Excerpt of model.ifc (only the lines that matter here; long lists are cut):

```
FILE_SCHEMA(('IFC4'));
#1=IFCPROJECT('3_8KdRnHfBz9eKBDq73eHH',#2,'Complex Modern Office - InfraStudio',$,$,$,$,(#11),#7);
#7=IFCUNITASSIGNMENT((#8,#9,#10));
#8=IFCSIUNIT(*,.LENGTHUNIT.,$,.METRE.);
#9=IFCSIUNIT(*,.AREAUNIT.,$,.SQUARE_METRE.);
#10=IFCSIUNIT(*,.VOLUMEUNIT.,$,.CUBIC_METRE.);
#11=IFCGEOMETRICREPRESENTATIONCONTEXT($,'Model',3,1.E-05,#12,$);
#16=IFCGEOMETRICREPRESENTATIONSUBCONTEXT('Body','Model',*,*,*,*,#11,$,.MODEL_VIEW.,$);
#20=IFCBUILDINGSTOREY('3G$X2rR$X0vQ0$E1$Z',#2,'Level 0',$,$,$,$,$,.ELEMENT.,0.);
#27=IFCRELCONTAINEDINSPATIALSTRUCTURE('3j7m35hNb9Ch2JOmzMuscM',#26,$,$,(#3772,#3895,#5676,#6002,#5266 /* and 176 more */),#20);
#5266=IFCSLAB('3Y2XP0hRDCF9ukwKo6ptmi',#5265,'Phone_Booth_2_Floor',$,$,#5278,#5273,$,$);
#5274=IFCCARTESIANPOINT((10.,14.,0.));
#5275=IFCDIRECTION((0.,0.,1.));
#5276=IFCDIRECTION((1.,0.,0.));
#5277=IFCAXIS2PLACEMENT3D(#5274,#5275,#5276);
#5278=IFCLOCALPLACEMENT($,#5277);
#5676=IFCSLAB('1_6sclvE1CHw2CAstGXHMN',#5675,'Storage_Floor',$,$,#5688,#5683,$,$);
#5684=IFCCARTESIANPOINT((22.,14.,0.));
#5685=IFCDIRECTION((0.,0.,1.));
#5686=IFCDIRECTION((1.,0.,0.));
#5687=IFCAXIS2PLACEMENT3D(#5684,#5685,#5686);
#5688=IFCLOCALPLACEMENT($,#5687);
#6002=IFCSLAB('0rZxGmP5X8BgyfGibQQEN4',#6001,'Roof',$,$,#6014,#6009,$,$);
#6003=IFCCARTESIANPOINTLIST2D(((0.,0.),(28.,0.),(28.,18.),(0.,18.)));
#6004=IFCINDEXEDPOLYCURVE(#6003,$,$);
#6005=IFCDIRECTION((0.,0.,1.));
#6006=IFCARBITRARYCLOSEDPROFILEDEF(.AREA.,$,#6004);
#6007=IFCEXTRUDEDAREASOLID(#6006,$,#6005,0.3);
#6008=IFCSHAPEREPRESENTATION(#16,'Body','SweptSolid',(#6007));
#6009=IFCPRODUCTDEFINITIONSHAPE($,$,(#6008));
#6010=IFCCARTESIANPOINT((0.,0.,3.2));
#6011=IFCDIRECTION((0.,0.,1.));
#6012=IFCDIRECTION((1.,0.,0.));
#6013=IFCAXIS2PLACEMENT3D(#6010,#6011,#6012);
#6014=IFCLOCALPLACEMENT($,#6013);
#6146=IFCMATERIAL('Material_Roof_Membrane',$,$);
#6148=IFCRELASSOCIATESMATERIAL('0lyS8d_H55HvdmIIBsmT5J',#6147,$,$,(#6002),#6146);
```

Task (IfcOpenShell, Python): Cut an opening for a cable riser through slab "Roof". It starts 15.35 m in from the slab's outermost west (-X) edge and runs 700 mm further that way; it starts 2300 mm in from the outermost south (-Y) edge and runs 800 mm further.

```python
import numpy as np
import ifcopenshell
import ifcopenshell.api.feature
import ifcopenshell.api.geometry
import ifcopenshell.api.root
import ifcopenshell.geom
import ifcopenshell.util.placement
import ifcopenshell.util.representation
import ifcopenshell.util.shape
import ifcopenshell.util.unit

model = ifcopenshell.open("model.ifc")
unit_scale = ifcopenshell.util.unit.calculate_unit_scale(model)
settings = ifcopenshell.geom.settings()


def volume(element):
    """Net volume in cubic metres, openings subtracted."""
    shape = ifcopenshell.geom.create_shape(settings, element)
    return ifcopenshell.util.shape.get_volume(shape.geometry)


slab = model.by_id(6002)
before = volume(slab)

# Extent in the slab's own axes, in metres. The edges named are its -X and -Y sides.
slab_shape = ifcopenshell.geom.create_shape(settings, slab)
vertices = ifcopenshell.util.shape.get_vertices(slab_shape.geometry)
x_min, y_min, bottom = vertices.min(axis=0)
top = vertices[:, 2].max()

opening = ifcopenshell.api.root.create_entity(model, ifc_class="IfcOpeningElement", name="Cable riser opening", predefined_type="OPENING")
context = ifcopenshell.util.representation.get_context(model, "Model", "Body", "MODEL_VIEW")
width, depth = 0.7, 0.8
outline = [(0.0, 0.0), (width, 0.0), (width, depth), (0.0, depth), (0.0, 0.0)]
# Overshoot both faces by 50 mm so the cut is clean.
shape = ifcopenshell.api.geometry.add_slab_representation(
    model, context=context, depth=top - bottom + 0.1, polyline=outline
)
ifcopenshell.api.geometry.assign_representation(model, product=opening, representation=shape)

matrix = ifcopenshell.util.placement.get_local_placement(slab.ObjectPlacement)
matrix[:, 3] = matrix @ np.append(np.array([x_min + 15.35, y_min + 2.3, bottom - 0.05]) / unit_scale, 1.0)
ifcopenshell.api.geometry.edit_object_placement(model, product=opening, matrix=matrix, is_si=False)
ifcopenshell.api.feature.add_feature(model, feature=opening, element=slab)

after = volume(slab)

print(f"slab volume {before:.3f} -> {after:.3f} m3")

model.write("model_updated.ifc")
```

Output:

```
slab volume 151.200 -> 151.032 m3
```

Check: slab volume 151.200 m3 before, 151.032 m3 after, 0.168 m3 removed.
